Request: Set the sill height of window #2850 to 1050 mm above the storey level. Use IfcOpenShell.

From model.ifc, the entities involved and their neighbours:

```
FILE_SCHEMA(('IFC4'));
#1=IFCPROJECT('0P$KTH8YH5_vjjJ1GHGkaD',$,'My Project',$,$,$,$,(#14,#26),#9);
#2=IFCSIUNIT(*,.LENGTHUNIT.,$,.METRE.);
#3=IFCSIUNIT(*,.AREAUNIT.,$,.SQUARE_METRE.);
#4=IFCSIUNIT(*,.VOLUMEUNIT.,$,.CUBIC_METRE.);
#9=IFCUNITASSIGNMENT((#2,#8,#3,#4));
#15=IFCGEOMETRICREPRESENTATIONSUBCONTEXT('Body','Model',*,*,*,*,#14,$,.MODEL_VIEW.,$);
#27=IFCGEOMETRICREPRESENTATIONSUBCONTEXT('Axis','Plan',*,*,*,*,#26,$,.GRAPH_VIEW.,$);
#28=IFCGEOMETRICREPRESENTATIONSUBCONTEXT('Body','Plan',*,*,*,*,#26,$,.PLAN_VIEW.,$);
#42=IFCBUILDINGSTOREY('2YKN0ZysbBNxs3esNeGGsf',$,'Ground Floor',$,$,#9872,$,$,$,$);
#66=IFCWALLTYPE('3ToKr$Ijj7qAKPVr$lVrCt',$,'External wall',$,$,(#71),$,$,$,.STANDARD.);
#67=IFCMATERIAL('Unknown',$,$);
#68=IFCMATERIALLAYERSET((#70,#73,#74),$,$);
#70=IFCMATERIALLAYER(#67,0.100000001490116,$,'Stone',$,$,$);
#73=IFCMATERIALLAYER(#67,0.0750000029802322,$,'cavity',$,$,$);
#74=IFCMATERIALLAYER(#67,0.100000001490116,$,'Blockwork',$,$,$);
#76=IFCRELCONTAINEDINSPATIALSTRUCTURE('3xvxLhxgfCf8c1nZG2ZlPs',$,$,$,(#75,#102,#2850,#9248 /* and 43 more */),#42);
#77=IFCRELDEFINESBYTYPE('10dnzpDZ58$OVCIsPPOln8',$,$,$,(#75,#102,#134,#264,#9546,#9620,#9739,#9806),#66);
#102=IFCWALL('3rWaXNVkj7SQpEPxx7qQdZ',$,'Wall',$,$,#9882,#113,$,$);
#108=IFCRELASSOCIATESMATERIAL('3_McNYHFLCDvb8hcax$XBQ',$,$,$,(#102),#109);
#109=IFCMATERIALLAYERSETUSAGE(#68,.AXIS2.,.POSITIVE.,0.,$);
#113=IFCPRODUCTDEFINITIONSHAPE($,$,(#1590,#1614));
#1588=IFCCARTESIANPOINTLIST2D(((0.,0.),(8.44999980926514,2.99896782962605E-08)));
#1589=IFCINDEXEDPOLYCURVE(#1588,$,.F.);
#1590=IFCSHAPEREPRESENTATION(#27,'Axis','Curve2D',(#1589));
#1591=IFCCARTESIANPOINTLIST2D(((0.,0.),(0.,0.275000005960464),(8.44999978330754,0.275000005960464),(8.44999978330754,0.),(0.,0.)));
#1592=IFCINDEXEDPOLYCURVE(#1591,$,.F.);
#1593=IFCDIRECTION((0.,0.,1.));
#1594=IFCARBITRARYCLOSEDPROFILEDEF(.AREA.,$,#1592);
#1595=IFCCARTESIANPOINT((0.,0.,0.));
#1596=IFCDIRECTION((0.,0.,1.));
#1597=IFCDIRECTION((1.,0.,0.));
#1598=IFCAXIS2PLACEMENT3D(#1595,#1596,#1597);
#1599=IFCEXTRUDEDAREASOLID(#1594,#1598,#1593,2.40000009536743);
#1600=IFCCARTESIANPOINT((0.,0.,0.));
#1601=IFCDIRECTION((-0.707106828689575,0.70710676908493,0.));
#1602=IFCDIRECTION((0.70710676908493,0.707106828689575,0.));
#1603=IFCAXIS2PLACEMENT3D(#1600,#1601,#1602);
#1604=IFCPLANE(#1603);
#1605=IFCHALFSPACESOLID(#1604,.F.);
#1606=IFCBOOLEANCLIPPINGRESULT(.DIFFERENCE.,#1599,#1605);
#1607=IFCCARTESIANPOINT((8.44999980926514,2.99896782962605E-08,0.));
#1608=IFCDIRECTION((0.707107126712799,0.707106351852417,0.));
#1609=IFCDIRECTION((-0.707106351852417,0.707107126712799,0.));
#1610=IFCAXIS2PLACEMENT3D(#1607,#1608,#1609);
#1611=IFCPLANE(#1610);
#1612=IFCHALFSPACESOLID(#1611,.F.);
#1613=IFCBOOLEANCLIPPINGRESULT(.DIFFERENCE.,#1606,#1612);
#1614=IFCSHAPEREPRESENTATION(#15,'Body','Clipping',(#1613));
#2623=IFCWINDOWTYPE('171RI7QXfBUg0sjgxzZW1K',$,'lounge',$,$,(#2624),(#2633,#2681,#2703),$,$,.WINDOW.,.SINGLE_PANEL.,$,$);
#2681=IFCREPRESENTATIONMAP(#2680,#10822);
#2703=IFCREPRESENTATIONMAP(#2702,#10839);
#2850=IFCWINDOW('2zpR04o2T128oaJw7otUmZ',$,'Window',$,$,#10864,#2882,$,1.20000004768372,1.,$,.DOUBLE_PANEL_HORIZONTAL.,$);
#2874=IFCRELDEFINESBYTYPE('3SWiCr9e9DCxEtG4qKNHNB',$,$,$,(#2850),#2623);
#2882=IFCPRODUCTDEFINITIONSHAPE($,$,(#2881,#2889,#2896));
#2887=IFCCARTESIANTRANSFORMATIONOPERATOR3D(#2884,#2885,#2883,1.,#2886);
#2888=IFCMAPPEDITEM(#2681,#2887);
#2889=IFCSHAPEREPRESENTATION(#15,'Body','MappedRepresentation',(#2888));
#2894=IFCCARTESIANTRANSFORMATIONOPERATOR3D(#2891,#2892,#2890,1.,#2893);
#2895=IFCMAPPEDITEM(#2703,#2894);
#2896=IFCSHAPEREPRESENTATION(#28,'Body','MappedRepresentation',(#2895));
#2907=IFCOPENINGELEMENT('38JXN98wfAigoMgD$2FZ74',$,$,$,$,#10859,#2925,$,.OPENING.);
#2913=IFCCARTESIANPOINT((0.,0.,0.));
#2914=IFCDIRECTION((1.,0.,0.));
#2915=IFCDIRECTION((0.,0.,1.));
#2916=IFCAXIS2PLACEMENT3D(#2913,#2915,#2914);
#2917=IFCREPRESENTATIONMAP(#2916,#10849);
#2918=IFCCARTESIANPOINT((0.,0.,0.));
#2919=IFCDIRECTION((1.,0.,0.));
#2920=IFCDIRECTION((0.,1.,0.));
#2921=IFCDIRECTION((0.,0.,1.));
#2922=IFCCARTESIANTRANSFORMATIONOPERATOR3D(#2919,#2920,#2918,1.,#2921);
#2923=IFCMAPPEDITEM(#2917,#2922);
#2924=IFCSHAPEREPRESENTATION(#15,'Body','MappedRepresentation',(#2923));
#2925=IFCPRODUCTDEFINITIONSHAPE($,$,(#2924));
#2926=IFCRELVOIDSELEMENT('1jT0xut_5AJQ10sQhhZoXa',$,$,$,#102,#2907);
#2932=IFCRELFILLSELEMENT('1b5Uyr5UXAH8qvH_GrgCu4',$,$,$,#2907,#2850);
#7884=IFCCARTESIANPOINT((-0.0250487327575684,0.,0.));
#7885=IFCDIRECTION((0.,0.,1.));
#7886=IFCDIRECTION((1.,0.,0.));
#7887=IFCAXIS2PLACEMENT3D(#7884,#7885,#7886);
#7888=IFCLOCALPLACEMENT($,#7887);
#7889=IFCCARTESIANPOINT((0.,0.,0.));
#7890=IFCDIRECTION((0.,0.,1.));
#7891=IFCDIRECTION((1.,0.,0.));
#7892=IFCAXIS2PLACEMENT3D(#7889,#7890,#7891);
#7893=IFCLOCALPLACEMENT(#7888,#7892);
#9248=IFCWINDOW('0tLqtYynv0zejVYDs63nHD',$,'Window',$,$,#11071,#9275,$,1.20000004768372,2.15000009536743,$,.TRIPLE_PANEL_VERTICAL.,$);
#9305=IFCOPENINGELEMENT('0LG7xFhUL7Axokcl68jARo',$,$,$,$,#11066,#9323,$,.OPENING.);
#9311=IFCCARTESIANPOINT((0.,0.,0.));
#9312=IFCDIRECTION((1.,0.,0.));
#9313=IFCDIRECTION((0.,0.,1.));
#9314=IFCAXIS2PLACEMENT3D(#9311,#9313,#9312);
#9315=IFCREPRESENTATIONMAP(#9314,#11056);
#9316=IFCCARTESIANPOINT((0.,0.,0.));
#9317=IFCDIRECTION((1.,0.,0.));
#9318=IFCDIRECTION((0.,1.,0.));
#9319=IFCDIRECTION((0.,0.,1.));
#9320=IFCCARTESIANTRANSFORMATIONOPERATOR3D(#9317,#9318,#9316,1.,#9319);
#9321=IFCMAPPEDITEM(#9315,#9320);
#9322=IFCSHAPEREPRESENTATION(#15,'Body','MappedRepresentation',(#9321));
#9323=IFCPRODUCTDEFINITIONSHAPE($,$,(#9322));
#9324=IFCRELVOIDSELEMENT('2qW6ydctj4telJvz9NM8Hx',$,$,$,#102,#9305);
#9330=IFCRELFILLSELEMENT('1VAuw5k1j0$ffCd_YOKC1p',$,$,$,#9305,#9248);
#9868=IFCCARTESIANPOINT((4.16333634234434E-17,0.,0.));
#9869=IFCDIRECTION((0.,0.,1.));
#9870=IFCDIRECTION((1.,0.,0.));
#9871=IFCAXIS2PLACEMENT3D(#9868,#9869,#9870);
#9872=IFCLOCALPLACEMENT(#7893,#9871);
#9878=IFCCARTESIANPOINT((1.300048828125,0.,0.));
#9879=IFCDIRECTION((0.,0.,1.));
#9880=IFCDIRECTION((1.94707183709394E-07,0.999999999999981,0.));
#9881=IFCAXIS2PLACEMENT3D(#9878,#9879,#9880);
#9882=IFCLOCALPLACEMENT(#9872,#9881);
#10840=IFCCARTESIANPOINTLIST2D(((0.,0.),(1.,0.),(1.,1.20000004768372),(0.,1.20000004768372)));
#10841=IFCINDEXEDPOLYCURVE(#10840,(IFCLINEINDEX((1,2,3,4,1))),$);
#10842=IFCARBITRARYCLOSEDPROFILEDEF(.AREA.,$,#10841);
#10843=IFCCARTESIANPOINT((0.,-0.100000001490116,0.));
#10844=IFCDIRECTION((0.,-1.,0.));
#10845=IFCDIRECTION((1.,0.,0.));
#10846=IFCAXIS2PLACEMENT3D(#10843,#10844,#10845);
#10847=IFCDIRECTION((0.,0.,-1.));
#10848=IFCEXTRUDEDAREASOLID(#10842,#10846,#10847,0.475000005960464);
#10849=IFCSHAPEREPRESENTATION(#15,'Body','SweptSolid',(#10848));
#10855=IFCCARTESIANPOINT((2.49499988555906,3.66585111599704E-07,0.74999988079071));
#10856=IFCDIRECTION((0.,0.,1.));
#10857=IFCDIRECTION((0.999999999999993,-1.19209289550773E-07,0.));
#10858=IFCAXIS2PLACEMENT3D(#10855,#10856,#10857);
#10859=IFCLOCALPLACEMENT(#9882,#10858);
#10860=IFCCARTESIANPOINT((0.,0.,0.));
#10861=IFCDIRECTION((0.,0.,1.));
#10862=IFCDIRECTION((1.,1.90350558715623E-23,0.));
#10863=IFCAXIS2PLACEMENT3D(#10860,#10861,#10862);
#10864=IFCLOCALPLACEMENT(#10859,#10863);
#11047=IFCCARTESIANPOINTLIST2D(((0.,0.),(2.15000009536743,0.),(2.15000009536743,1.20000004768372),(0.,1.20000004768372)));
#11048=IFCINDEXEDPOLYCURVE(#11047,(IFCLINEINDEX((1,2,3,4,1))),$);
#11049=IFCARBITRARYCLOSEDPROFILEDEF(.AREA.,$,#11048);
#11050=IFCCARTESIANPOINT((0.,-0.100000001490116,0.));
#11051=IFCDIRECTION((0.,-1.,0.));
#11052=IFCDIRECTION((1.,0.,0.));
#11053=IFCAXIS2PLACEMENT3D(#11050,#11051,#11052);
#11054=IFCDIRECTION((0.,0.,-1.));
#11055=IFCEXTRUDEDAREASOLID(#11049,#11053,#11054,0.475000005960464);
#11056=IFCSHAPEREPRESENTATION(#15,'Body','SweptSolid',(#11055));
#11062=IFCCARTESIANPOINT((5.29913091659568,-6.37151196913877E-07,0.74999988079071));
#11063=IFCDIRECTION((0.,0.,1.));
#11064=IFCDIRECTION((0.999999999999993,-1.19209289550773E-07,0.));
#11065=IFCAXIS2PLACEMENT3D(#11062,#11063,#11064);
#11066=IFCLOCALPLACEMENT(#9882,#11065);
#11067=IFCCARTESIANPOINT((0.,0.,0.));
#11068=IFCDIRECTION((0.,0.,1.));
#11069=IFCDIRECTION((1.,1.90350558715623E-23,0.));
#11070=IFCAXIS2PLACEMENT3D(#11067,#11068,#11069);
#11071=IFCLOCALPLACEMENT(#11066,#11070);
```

```python
import numpy as np
import ifcopenshell
import ifcopenshell.api.geometry
import ifcopenshell.geom
import ifcopenshell.util.element
import ifcopenshell.util.placement
import ifcopenshell.util.shape
import ifcopenshell.util.unit

model = ifcopenshell.open("model.ifc")
unit_scale = ifcopenshell.util.unit.calculate_unit_scale(model)

window = model.by_guid("2zpR04o2T128oaJw7otUmZ")
opening = window.FillsVoids[0].RelatingOpeningElement
storey = ifcopenshell.util.element.get_container(window, ifc_class="IfcBuildingStorey")
level = ifcopenshell.util.placement.get_local_placement(storey.ObjectPlacement)[2, 3]

# The opening's origin need not be at the sill, so measure its lowest point.
shape = ifcopenshell.geom.create_shape(ifcopenshell.geom.settings(), opening)
bottom = ifcopenshell.util.shape.get_shape_bottom_elevation(shape, shape.geometry) / unit_scale
dz = level + 1.05 / unit_scale - bottom

shift = np.array([0.0, 0.0, dz])
# The window is placed relative to its opening, so it follows when the opening moves.
matrix = ifcopenshell.util.placement.get_local_placement(opening.ObjectPlacement)
matrix[:3, 3] += shift
ifcopenshell.api.geometry.edit_object_placement(
    model, product=opening, matrix=matrix, is_si=False, should_transform_children=True
)

print(f"moved by {dz * unit_scale:+.3f} m")

model.write("model-out.ifc")
```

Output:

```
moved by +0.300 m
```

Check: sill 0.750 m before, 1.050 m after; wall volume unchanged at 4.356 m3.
